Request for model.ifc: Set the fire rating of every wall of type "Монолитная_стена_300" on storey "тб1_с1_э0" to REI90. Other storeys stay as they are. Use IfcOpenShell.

First a look at what the model holds.

```python
import ifcopenshell
import ifcopenshell.util.element

model = ifcopenshell.open("model.ifc")
print(model.schema)
storey = next(s for s in model.by_type("IfcBuildingStorey") if s.Name == "тб1_с1_э0")
walls = [e for e in ifcopenshell.util.element.get_decomposition(storey) if e.is_a("IfcWall")]
seen = {}
for e in walls:
    element_type = ifcopenshell.util.element.get_type(e)
    key = (element_type.Name if element_type != e and element_type else None, ifcopenshell.util.element.get_pset(e, "Pset_WallCommon", "FireRating"))
    seen[key] = seen.get(key, 0) + 1
for (name, value), count in sorted(seen.items(), key=str):
    print(count, "x", name, "|", value)
```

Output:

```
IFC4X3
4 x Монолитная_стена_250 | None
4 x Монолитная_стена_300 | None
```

```python
import ifcopenshell
import ifcopenshell.api.pset
import ifcopenshell.util.element

model = ifcopenshell.open("model.ifc")

storey = next(s for s in model.by_type("IfcBuildingStorey") if s.Name == "тб1_с1_э0")
walls = [e for e in ifcopenshell.util.element.get_decomposition(storey) if e.is_a("IfcWall")]

count = 0
for e in walls:
    element_type = ifcopenshell.util.element.get_type(e)
    if element_type in (None, e) or element_type.Name != "Монолитная_стена_300":
        continue
    # add_pset returns the element's existing set when there is one.
    pset = ifcopenshell.api.pset.add_pset(model, product=e, name="Pset_WallCommon")
    ifcopenshell.api.pset.edit_pset(model, pset=pset, properties={"FireRating": "REI90"})
    count += 1

print(count, "walls updated")

model.write("model-out.ifc")
```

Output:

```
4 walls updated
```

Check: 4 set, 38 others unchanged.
